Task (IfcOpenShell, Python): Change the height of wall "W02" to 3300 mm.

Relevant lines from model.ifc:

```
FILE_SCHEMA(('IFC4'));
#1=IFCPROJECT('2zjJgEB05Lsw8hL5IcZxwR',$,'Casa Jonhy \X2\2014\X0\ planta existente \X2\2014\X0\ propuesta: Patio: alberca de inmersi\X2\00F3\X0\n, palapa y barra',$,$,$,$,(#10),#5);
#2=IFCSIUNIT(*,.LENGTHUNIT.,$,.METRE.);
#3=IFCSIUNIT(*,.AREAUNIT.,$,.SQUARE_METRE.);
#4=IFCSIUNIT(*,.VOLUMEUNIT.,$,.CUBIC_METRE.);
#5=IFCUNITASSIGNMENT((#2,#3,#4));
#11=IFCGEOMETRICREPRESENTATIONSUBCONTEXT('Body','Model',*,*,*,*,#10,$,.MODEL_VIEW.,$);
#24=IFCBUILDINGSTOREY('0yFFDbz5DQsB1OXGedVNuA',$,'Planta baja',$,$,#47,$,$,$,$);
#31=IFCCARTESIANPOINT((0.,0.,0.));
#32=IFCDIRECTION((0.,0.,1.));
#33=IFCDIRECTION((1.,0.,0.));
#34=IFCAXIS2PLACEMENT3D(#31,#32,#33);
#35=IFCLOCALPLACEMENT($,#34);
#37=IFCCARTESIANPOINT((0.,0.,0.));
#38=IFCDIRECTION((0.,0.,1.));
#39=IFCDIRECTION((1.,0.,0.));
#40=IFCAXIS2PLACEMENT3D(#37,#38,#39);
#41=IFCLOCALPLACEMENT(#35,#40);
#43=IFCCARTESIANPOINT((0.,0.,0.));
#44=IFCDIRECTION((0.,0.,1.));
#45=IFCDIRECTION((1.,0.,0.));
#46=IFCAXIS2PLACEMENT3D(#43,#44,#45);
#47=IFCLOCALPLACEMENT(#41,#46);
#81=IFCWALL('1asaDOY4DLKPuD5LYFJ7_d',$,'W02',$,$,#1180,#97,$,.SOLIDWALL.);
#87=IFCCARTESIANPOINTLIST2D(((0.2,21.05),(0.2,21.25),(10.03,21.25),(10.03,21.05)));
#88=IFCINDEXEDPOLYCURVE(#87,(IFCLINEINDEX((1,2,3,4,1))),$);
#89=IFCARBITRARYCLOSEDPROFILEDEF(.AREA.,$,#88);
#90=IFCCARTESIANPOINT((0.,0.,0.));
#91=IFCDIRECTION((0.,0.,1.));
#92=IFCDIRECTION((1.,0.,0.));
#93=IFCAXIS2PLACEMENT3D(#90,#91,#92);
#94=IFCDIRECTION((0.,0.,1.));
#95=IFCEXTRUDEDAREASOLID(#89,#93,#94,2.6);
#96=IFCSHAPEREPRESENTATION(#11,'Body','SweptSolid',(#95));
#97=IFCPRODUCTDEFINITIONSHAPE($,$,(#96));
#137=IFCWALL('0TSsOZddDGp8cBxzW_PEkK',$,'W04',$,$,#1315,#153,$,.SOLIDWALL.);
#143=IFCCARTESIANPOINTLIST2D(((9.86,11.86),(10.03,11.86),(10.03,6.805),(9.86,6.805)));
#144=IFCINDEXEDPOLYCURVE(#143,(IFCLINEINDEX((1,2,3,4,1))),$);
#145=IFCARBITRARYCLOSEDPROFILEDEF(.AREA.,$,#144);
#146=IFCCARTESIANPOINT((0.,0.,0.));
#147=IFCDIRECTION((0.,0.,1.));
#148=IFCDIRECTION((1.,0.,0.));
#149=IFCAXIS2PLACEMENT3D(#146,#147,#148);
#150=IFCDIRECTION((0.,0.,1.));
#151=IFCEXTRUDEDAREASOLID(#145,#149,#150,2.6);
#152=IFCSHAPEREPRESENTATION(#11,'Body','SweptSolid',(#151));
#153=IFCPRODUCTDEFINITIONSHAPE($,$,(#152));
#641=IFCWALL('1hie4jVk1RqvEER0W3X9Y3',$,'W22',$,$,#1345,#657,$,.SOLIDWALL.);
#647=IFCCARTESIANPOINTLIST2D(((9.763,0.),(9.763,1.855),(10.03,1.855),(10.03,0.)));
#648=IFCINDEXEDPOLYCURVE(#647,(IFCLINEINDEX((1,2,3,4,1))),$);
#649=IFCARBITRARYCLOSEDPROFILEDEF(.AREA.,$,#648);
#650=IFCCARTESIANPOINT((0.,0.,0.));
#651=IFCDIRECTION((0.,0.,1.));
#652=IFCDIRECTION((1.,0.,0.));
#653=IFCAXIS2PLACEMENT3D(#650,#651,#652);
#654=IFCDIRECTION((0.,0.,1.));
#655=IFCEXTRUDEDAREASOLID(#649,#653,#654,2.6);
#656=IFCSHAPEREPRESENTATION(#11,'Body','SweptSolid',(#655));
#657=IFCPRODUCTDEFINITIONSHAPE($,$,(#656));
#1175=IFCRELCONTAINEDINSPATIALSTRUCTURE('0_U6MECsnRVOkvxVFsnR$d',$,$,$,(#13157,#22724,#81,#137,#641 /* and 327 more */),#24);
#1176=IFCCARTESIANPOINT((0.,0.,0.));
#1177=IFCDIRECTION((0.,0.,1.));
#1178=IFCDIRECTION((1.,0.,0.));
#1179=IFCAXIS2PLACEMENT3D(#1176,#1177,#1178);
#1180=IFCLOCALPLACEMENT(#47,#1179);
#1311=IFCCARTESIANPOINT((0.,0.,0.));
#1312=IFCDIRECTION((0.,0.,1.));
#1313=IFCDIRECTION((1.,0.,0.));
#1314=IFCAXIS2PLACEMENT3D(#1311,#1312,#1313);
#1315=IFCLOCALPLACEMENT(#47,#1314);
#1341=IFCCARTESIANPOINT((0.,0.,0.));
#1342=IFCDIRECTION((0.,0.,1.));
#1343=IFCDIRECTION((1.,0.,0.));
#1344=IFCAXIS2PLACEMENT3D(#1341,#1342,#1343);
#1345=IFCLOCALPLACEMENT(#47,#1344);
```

```python
import ifcopenshell
import ifcopenshell.geom
import ifcopenshell.util.representation
import ifcopenshell.util.shape

model = ifcopenshell.open("model.ifc")
settings = ifcopenshell.geom.settings()


def volume(element):
    """Net volume in cubic metres, openings subtracted."""
    shape = ifcopenshell.geom.create_shape(settings, element)
    return ifcopenshell.util.shape.get_volume(shape.geometry)


wall = model.by_guid("1asaDOY4DLKPuD5LYFJ7_d")
before = volume(wall)

body = ifcopenshell.util.representation.get_representation(wall, "Model", "Body")
solid = body.Items[0]
old_height = solid.Depth
solid.Depth = 3.3
after = volume(wall)

print(f"height {old_height:g} -> {solid.Depth:g}, volume {before:.3f} -> {after:.3f} m3")

model.write("model-out.ifc")
```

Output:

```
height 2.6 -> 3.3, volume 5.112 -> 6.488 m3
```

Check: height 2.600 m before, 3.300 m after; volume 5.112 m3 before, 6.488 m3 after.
